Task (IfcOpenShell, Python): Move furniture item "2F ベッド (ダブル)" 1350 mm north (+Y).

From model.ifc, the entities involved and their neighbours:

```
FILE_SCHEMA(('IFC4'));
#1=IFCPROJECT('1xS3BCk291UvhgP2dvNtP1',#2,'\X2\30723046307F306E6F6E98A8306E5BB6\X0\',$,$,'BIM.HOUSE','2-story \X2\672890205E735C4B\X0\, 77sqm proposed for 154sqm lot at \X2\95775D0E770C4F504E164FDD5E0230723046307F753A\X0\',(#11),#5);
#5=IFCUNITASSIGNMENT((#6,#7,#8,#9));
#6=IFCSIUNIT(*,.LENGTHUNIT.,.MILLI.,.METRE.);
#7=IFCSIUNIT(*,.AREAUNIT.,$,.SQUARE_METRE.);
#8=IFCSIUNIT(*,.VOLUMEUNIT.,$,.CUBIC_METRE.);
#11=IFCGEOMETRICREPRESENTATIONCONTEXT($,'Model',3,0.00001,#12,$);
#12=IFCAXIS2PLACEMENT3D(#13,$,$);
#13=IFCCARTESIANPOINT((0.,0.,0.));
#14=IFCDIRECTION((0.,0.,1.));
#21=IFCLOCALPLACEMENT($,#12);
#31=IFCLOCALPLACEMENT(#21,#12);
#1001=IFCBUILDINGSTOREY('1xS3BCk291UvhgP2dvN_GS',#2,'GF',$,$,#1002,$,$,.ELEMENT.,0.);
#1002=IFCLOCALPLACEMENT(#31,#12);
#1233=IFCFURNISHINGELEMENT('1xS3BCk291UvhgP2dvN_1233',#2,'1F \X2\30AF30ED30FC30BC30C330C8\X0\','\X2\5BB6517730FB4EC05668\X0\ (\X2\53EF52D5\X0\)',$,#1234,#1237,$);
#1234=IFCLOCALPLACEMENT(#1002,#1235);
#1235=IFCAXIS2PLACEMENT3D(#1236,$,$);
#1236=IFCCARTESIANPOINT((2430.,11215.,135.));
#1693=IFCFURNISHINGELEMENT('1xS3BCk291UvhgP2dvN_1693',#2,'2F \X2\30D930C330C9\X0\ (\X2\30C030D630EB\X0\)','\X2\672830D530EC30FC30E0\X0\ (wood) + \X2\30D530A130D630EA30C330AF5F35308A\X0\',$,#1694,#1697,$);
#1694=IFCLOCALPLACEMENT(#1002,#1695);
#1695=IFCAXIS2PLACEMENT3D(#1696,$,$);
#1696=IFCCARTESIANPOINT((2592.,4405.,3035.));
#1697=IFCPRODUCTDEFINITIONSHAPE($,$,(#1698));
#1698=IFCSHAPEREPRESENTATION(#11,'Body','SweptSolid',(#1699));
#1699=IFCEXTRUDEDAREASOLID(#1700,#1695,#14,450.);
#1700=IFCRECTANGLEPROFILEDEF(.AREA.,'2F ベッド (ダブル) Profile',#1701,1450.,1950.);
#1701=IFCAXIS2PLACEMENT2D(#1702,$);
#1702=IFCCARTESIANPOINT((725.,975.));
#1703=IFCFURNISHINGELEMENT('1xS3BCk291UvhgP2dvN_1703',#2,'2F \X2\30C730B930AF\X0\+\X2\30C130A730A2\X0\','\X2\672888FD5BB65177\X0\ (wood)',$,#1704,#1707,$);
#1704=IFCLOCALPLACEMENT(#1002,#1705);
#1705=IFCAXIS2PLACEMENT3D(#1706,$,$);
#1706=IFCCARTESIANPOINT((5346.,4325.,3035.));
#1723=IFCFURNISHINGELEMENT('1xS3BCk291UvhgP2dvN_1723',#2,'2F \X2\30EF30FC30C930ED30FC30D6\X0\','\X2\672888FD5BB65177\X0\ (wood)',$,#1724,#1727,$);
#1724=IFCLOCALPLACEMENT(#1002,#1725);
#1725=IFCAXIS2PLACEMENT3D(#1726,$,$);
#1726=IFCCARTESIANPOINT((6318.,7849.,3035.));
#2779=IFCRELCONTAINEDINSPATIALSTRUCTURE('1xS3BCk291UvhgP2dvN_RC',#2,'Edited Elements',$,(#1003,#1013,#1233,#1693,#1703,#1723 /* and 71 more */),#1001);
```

```python
import ifcopenshell
import ifcopenshell.api.geometry
import ifcopenshell.util.placement
import ifcopenshell.util.unit

model = ifcopenshell.open("model.ifc")
unit_scale = ifcopenshell.util.unit.calculate_unit_scale(model)

item = model.by_guid("1xS3BCk291UvhgP2dvN_1693")
matrix = ifcopenshell.util.placement.get_local_placement(item.ObjectPlacement)
matrix[1, 3] += 1.35 / unit_scale
ifcopenshell.api.geometry.edit_object_placement(model, product=item, matrix=matrix, is_si=False)

print(ifcopenshell.util.placement.get_local_placement(item.ObjectPlacement).round(3) + 0.0)

model.write("model_v2.ifc")
```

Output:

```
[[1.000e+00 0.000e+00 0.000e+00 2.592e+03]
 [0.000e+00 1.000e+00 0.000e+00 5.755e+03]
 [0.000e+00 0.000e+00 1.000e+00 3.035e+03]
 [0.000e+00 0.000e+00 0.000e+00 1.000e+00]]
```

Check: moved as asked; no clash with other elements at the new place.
